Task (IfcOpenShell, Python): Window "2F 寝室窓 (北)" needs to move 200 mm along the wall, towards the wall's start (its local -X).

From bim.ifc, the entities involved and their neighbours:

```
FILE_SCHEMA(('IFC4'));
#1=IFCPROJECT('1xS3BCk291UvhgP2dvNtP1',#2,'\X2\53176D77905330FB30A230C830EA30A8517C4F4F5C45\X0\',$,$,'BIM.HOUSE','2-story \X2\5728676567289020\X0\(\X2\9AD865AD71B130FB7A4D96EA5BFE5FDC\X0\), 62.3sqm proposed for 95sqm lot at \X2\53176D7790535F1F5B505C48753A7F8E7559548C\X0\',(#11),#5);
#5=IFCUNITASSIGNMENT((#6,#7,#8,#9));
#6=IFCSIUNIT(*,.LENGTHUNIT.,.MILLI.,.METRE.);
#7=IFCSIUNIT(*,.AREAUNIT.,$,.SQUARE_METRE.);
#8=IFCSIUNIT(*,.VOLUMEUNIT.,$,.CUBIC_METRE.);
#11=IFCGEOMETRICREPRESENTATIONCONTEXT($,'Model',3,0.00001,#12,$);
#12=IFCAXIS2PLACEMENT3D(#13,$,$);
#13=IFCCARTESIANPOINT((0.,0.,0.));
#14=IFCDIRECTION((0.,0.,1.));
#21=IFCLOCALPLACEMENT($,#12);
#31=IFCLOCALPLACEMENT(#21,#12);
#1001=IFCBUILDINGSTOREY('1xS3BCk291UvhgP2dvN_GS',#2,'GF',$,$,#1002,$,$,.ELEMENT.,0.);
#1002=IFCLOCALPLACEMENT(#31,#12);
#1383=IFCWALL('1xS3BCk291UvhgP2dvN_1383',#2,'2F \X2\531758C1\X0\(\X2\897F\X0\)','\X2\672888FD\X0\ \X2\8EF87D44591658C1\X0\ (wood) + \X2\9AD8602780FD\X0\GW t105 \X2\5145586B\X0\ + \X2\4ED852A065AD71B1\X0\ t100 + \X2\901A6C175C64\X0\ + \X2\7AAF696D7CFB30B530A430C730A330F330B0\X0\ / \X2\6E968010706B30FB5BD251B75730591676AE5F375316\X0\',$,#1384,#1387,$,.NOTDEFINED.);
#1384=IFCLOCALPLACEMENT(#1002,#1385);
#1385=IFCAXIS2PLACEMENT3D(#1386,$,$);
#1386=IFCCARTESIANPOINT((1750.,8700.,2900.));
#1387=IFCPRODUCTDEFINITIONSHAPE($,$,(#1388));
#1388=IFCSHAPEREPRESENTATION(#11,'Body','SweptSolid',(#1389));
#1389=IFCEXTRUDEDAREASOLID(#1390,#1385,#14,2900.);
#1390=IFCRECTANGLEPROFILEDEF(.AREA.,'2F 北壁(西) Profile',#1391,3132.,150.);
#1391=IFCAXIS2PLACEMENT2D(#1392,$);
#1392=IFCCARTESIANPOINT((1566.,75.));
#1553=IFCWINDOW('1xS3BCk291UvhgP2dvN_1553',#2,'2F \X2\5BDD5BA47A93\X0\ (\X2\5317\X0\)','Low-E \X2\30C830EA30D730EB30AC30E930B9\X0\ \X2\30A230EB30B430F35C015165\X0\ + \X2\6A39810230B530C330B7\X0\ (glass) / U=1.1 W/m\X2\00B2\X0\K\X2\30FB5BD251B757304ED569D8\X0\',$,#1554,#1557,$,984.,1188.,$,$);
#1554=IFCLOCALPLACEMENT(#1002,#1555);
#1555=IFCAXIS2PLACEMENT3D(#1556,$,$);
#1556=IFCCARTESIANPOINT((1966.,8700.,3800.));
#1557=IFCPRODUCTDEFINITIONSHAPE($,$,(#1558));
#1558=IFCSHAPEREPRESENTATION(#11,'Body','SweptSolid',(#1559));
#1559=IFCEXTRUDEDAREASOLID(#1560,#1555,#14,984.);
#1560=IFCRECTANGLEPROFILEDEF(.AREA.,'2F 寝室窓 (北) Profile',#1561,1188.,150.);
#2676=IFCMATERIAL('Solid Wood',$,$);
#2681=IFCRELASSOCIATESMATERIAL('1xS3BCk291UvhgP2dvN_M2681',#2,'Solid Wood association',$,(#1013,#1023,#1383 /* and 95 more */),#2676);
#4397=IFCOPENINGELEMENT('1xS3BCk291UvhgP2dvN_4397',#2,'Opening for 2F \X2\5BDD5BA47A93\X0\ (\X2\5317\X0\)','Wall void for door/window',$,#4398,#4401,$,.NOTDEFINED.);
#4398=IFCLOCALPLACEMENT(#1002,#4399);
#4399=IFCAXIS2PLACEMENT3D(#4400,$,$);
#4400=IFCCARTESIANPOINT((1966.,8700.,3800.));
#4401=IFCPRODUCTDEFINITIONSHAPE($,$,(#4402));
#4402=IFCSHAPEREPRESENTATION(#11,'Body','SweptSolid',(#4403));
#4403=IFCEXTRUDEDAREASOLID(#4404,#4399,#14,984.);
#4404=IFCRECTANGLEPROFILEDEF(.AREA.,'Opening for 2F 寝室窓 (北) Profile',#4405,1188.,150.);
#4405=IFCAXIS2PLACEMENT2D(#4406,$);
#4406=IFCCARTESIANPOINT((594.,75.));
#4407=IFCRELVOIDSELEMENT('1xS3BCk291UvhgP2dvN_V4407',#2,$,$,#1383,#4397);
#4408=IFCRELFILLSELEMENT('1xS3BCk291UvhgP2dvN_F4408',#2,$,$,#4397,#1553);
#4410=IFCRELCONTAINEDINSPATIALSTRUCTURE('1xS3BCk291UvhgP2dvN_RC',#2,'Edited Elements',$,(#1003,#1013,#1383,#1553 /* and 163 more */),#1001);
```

```python
import ifcopenshell
import ifcopenshell.api.geometry
import ifcopenshell.util.placement
import ifcopenshell.util.unit

model = ifcopenshell.open("bim.ifc")
unit_scale = ifcopenshell.util.unit.calculate_unit_scale(model)

window = model.by_guid("1xS3BCk291UvhgP2dvN_1553")
opening = window.FillsVoids[0].RelatingOpeningElement
wall = opening.VoidsElements[0].RelatingBuildingElement

wall_matrix = ifcopenshell.util.placement.get_local_placement(wall.ObjectPlacement)
shift = wall_matrix[:3, 0] * -0.2 / unit_scale
before = ifcopenshell.util.placement.get_local_placement(window.ObjectPlacement)[:3, 3].copy()

# The window is not placed relative to its opening, so move both.
for product in (opening, window):
    matrix = ifcopenshell.util.placement.get_local_placement(product.ObjectPlacement)
    matrix[:3, 3] += shift
    ifcopenshell.api.geometry.edit_object_placement(model, product=product, matrix=matrix, is_si=False)

after = ifcopenshell.util.placement.get_local_placement(window.ObjectPlacement)[:3, 3]
print("window moved by", (after - before).round(3) + 0.0)

model.write("bim_rev.ifc")
```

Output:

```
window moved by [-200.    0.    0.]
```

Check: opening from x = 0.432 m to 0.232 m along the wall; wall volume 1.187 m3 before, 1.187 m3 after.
